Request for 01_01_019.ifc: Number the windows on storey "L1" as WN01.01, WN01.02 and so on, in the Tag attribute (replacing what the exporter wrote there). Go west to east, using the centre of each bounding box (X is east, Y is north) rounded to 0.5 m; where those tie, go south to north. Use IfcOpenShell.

First a look at what the model holds.

```python
import ifcopenshell
import ifcopenshell.util.element
import ifcopenshell.util.placement

model = ifcopenshell.open("01_01_019.ifc")
print(model.schema)
storey = next(s for s in model.by_type("IfcBuildingStorey") if s.Name == "L1")
windows = [e for e in ifcopenshell.util.element.get_decomposition(storey) if e.is_a("IfcWindow")]
for e in sorted(windows, key=lambda e: e.id()):
    origin = ifcopenshell.util.placement.get_local_placement(e.ObjectPlacement)[:3, 3]
    print(e.id(), e.Tag, e.Name, origin.round(2) + 0.0, sep=" | ")
```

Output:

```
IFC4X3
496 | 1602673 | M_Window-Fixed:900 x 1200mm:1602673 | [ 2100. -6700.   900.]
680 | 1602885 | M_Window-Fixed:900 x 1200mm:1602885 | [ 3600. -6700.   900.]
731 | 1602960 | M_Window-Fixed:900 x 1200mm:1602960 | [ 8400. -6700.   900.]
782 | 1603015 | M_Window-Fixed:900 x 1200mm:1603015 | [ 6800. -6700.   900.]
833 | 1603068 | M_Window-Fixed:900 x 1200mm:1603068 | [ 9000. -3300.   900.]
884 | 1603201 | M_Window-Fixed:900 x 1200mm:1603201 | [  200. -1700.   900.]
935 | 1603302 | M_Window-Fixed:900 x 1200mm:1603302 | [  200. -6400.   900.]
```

```python
import ifcopenshell
import ifcopenshell.geom
import ifcopenshell.util.element
import ifcopenshell.util.shape

model = ifcopenshell.open("01_01_019.ifc")
settings = ifcopenshell.geom.settings()
settings.set("use-world-coords", True)


def centre(element):
    shape = ifcopenshell.geom.create_shape(settings, element)
    return ifcopenshell.util.shape.get_bbox_centroid(shape.geometry)


storey = next(s for s in model.by_type("IfcBuildingStorey") if s.Name == "L1")
windows = [e for e in ifcopenshell.util.element.get_decomposition(storey) if e.is_a("IfcWindow")]

# Insertion points can sit at a corner or the storey origin, so sort by the geometry (in metres).
centres = {e: centre(e) for e in windows}
windows.sort(key=lambda e: (round(centres[e][0] / 0.5), centres[e][1]))

for i, e in enumerate(windows, start=1):
    number = f"WN01.{i:02d}"
    e.Tag = number
    print(e.id(), number)

model.write("01_01_019_v2.ifc")
```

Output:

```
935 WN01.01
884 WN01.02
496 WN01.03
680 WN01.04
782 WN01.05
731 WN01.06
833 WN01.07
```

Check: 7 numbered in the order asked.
